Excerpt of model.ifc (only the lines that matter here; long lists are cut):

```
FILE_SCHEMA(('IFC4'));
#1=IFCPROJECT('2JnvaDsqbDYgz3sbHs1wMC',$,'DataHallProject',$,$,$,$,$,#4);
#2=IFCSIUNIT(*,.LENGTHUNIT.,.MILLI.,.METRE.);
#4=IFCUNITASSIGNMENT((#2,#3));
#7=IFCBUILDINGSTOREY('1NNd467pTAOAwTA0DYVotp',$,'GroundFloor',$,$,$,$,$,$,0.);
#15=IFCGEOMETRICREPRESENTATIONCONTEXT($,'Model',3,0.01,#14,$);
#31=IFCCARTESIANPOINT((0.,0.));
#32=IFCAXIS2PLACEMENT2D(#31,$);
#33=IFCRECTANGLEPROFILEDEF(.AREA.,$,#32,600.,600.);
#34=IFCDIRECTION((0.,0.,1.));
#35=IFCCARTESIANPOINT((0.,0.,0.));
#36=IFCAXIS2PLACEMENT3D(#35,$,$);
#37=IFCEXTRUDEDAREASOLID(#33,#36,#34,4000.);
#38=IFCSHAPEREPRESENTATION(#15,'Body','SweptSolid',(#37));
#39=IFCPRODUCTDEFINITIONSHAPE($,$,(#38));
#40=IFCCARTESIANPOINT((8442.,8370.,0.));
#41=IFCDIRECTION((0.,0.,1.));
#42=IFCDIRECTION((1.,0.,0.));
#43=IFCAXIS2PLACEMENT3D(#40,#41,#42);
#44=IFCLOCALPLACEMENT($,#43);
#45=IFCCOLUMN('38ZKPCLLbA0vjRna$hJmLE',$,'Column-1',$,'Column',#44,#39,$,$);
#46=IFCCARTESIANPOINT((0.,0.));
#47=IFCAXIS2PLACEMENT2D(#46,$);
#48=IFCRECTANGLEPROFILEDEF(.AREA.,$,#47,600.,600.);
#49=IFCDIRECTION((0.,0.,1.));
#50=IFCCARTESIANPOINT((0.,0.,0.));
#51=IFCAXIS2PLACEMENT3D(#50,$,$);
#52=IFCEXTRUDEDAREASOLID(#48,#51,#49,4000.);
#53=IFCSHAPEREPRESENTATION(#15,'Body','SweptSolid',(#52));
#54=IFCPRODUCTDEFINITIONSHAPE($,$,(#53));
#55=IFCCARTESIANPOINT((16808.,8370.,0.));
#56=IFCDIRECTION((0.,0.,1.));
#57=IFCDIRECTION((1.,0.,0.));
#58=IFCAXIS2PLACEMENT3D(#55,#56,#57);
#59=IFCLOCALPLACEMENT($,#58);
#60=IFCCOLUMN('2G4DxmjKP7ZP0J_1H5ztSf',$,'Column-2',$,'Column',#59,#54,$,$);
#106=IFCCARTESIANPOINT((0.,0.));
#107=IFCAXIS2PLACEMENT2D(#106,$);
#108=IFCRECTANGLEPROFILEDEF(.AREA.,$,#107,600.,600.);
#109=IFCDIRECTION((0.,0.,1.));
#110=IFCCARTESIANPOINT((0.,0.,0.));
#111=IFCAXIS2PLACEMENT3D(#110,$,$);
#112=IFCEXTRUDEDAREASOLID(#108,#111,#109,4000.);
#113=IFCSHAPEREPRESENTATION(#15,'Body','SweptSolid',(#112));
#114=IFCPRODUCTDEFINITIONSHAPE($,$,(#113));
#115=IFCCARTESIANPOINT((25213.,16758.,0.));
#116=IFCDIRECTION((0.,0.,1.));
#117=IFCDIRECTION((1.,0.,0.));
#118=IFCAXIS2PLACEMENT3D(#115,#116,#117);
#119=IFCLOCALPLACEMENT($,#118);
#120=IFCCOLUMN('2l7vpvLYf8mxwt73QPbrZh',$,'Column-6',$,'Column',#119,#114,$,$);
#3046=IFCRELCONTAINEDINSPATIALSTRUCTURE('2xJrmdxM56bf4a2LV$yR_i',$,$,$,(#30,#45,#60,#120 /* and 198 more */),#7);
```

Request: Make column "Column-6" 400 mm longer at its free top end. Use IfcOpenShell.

```python
import ifcopenshell

model = ifcopenshell.open("model.ifc")

member = model.by_id(120)
change = 400.0

# The extrusion runs towards the end named, so only its depth changes.
body = next(r for r in member.Representation.Representations if r.RepresentationIdentifier == "Body")
solid = body.Items[0]
old_length = solid.Depth
solid.Depth += change

print(f"length {old_length:g} -> {solid.Depth:g}")

model.write("model_edited.ifc")
```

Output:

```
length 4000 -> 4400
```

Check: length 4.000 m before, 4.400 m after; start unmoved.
